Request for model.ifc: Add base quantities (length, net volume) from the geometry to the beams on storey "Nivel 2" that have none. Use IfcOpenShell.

First a look at what the model holds.

```python
import ifcopenshell
import ifcopenshell.util.element
import ifcopenshell.util.unit

model = ifcopenshell.open("model.ifc")
print(model.schema)
for unit_type in ("LENGTHUNIT", "AREAUNIT", "VOLUMEUNIT"):
    print(unit_type, ifcopenshell.util.unit.calculate_unit_scale(model, unit_type))
storey = next(s for s in model.by_type("IfcBuildingStorey") if s.Name == "Nivel 2")
beams = [e for e in ifcopenshell.util.element.get_decomposition(storey) if e.is_a("IfcBeam")]
for e in sorted(beams, key=lambda e: e.id()):
    print(e.id(), e.is_a(), e.Name, list(ifcopenshell.util.element.get_psets(e, qtos_only=True)), sep=" | ")
```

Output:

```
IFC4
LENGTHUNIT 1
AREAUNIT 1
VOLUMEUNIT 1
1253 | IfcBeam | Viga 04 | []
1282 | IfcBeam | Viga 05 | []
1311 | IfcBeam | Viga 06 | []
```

```python
import ifcopenshell
import ifcopenshell.api.pset
import ifcopenshell.geom
import ifcopenshell.util.element
import ifcopenshell.util.shape
import ifcopenshell.util.unit

model = ifcopenshell.open("model.ifc")
unit_scale = ifcopenshell.util.unit.calculate_unit_scale(model)
volume_scale = ifcopenshell.util.unit.calculate_unit_scale(model, "VOLUMEUNIT")
settings = ifcopenshell.geom.settings()

storey = next(s for s in model.by_type("IfcBuildingStorey") if s.Name == "Nivel 2")
beams = [e for e in ifcopenshell.util.element.get_decomposition(storey) if e.is_a("IfcBeam")]

for e in sorted(beams, key=lambda e: e.id()):
    if ifcopenshell.util.element.get_psets(e, qtos_only=True, should_inherit=False):
        continue
    # Geometry comes back in metres, in the element's own axes.
    shape = ifcopenshell.geom.create_shape(settings, e)
    values = {
        "Length": ifcopenshell.util.shape.get_max_xyz(shape.geometry) / unit_scale,
        "NetVolume": ifcopenshell.util.shape.get_volume(shape.geometry) / volume_scale,
    }
    qto = ifcopenshell.api.pset.add_qto(model, product=e, name="Qto_BeamBaseQuantities")
    ifcopenshell.api.pset.edit_qto(model, qto=qto, properties=values)
    print(e.id(), {k: round(v, 3) for k, v in values.items()})

model.write("model-out.ifc")
```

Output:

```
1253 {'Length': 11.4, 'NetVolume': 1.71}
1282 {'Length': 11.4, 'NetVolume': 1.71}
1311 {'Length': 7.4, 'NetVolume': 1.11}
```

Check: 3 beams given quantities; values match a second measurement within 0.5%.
